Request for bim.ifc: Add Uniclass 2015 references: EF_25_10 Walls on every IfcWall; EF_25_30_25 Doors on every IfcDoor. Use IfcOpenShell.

First a look at what the model holds.

```python
import ifcopenshell

model = ifcopenshell.open("bim.ifc")
print(model.schema)
print("classifications:", [c.Name for c in model.by_type("IfcClassification")])
for ifc_class in ("IfcDoor", "IfcRoof", "IfcStair", "IfcWall", "IfcWindow"):
    print(ifc_class, len(model.by_type(ifc_class)))
```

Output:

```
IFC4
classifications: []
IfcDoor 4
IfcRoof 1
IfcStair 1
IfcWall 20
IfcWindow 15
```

```python
import ifcopenshell
import ifcopenshell.api.classification

model = ifcopenshell.open("bim.ifc")

system = ifcopenshell.api.classification.add_classification(model, classification="Uniclass 2015")

codes = {
    "IfcWall": ("EF_25_10", "Walls"),
    "IfcDoor": ("EF_25_30_25", "Doors"),
}
for ifc_class, (code, name) in codes.items():
    products = model.by_type(ifc_class)
    ifcopenshell.api.classification.add_reference(
        model, products=products, classification=system, identification=code, name=name
    )
    print(code, len(products))

model.write("bim_edited.ifc")
```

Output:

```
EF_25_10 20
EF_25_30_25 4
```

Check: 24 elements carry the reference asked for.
